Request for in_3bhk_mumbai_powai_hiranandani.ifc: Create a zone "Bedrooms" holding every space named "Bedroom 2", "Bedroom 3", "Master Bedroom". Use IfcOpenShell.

First a look at what the model holds.

```python
import ifcopenshell

model = ifcopenshell.open("in_3bhk_mumbai_powai_hiranandani.ifc")
print(model.schema)
seen = {}
for space in model.by_type("IfcSpace"):
    seen[space.LongName] = seen.get(space.LongName, 0) + 1
for name, count in sorted(seen.items(), key=str):
    print(count, "x", name)
print("zones:", [z.Name for z in model.by_type("IfcZone")][:20])
```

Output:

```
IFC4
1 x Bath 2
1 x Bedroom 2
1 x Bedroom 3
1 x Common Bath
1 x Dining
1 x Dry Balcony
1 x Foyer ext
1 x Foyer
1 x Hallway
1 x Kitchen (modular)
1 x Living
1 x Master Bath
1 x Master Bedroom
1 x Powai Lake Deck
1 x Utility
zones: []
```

```python
import ifcopenshell
import ifcopenshell.api.group
import ifcopenshell.api.root

model = ifcopenshell.open("in_3bhk_mumbai_powai_hiranandani.ifc")

names = {"Bedroom 2", "Bedroom 3", "Master Bedroom"}
spaces = [s for s in model.by_type("IfcSpace") if s.LongName in names]

zone = ifcopenshell.api.root.create_entity(model, ifc_class="IfcZone", name="Bedrooms")
ifcopenshell.api.group.assign_group(model, products=spaces, group=zone)
print(len(spaces), "spaces in", zone.Name)

model.write("in_3bhk_mumbai_powai_hiranandani_updated.ifc")
```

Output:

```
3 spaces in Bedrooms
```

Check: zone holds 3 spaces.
